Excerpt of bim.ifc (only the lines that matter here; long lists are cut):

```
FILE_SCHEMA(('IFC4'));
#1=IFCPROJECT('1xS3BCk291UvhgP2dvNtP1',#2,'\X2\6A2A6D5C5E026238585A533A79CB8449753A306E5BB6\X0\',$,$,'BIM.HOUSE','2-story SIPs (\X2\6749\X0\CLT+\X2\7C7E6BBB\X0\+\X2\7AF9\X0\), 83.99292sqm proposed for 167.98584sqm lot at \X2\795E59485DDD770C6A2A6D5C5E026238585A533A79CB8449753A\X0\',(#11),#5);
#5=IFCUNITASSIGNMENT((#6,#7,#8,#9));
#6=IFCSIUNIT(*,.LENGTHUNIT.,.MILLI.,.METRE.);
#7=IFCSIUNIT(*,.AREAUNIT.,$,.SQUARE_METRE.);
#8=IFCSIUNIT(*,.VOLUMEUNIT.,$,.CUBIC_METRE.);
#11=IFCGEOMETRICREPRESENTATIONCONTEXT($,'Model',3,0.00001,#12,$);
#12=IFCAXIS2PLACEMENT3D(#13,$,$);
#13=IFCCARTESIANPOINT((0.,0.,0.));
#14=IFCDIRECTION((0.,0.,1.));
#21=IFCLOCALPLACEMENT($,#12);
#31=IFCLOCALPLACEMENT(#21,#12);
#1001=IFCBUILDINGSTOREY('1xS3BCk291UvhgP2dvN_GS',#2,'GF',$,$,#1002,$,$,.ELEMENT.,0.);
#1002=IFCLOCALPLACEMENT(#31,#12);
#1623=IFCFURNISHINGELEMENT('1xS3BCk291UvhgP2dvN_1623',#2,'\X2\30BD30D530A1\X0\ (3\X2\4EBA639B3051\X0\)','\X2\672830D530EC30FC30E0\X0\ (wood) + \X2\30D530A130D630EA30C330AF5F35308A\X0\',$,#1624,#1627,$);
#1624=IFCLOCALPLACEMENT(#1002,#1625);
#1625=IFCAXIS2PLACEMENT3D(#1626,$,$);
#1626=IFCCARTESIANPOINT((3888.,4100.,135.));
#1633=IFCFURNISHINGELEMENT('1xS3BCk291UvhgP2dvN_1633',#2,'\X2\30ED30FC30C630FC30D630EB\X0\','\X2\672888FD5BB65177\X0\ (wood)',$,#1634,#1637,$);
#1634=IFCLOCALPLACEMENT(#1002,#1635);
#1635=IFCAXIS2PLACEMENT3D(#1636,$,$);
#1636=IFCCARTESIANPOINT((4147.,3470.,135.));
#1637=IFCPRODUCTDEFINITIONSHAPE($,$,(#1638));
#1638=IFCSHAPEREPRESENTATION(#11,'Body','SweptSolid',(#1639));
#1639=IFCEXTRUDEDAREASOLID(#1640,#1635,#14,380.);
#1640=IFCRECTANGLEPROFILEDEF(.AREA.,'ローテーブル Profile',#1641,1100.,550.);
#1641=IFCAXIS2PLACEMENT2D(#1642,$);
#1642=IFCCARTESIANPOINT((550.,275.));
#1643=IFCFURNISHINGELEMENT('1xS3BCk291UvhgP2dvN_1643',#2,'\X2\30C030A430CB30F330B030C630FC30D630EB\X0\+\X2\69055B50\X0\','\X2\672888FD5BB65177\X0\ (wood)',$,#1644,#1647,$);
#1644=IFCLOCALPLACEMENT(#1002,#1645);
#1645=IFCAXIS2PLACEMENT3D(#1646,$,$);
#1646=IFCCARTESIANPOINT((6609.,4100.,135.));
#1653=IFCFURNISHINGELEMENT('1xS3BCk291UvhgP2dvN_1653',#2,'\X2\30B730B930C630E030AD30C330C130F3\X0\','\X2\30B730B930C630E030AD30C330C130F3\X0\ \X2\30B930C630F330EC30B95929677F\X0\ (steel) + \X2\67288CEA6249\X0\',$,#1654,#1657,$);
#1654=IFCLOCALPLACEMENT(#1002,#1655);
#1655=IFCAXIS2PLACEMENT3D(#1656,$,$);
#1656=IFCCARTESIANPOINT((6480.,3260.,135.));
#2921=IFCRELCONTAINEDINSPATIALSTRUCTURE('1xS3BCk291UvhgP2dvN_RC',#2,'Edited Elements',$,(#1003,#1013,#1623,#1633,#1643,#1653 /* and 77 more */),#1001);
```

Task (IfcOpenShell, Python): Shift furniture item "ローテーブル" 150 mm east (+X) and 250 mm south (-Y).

```python
import ifcopenshell
import ifcopenshell.api.geometry
import ifcopenshell.util.placement

model = ifcopenshell.open("bim.ifc")

item = model.by_guid("1xS3BCk291UvhgP2dvN_1633")
matrix = ifcopenshell.util.placement.get_local_placement(item.ObjectPlacement)
matrix[0, 3] += 150.0
matrix[1, 3] -= 250.0
ifcopenshell.api.geometry.edit_object_placement(model, product=item, matrix=matrix, is_si=False)

print(ifcopenshell.util.placement.get_local_placement(item.ObjectPlacement).round(3) + 0.0)

model.write("bim-out.ifc")
```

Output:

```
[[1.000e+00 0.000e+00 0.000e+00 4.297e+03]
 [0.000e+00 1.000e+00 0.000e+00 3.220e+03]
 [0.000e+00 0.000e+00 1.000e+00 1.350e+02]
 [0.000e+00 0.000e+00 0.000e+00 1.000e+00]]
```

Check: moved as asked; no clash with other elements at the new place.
